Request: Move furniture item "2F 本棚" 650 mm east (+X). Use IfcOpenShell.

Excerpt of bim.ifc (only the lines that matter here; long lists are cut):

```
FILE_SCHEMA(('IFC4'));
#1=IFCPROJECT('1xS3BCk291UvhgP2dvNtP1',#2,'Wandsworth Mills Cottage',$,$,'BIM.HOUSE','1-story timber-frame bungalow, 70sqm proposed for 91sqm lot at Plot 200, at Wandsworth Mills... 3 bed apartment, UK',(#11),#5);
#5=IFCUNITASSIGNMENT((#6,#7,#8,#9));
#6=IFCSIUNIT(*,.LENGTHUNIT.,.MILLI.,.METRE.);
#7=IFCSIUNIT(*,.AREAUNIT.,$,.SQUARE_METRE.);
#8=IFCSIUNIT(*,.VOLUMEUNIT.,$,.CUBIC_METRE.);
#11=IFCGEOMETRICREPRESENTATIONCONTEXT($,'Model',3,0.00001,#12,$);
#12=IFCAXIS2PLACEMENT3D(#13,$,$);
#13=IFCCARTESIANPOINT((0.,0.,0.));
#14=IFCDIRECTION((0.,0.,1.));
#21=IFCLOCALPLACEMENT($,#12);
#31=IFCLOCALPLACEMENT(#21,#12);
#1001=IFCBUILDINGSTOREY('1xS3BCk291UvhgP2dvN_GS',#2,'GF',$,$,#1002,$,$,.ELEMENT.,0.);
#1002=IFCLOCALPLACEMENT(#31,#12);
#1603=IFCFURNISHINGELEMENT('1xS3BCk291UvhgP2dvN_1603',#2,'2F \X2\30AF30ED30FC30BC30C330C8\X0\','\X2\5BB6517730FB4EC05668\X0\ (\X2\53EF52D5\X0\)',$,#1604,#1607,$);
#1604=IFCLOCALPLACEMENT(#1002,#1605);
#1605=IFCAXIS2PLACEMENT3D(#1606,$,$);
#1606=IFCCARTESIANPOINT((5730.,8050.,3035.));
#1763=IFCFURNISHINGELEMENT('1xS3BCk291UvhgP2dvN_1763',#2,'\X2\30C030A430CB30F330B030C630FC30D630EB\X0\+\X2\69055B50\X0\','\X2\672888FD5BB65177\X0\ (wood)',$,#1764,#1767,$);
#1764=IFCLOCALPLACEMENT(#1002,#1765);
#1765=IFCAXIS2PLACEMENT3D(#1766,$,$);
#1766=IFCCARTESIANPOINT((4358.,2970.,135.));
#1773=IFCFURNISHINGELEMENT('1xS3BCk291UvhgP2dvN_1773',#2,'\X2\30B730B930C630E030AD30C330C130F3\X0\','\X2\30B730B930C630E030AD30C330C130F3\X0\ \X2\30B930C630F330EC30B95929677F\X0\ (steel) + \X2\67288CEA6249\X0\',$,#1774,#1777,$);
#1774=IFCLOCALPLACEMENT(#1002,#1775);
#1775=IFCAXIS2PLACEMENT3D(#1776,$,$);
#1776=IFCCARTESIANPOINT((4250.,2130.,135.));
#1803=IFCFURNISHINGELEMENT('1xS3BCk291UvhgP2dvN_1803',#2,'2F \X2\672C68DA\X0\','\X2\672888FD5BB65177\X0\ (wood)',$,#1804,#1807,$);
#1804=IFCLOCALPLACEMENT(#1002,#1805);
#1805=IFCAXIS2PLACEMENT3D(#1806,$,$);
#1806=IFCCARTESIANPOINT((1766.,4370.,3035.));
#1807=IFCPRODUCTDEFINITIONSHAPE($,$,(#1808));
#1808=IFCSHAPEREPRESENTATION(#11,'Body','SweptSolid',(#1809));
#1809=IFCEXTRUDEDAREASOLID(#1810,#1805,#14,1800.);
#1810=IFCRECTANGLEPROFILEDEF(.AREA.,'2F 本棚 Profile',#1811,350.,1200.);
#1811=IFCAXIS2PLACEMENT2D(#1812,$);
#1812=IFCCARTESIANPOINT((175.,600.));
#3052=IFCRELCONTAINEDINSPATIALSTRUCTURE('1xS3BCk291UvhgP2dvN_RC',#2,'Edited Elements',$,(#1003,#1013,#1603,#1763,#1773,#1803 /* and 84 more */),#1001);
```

```python
import ifcopenshell
import ifcopenshell.api.geometry
import ifcopenshell.util.placement
import ifcopenshell.util.unit

model = ifcopenshell.open("bim.ifc")
unit_scale = ifcopenshell.util.unit.calculate_unit_scale(model)

item = model.by_guid("1xS3BCk291UvhgP2dvN_1803")
matrix = ifcopenshell.util.placement.get_local_placement(item.ObjectPlacement)
matrix[0, 3] += 0.65 / unit_scale
ifcopenshell.api.geometry.edit_object_placement(model, product=item, matrix=matrix, is_si=False)

print(ifcopenshell.util.placement.get_local_placement(item.ObjectPlacement).round(3) + 0.0)

model.write("bim-out.ifc")
```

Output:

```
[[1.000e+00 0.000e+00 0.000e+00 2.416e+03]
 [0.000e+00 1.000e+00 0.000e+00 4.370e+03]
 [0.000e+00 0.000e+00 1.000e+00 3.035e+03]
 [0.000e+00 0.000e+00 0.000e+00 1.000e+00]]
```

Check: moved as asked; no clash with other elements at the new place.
